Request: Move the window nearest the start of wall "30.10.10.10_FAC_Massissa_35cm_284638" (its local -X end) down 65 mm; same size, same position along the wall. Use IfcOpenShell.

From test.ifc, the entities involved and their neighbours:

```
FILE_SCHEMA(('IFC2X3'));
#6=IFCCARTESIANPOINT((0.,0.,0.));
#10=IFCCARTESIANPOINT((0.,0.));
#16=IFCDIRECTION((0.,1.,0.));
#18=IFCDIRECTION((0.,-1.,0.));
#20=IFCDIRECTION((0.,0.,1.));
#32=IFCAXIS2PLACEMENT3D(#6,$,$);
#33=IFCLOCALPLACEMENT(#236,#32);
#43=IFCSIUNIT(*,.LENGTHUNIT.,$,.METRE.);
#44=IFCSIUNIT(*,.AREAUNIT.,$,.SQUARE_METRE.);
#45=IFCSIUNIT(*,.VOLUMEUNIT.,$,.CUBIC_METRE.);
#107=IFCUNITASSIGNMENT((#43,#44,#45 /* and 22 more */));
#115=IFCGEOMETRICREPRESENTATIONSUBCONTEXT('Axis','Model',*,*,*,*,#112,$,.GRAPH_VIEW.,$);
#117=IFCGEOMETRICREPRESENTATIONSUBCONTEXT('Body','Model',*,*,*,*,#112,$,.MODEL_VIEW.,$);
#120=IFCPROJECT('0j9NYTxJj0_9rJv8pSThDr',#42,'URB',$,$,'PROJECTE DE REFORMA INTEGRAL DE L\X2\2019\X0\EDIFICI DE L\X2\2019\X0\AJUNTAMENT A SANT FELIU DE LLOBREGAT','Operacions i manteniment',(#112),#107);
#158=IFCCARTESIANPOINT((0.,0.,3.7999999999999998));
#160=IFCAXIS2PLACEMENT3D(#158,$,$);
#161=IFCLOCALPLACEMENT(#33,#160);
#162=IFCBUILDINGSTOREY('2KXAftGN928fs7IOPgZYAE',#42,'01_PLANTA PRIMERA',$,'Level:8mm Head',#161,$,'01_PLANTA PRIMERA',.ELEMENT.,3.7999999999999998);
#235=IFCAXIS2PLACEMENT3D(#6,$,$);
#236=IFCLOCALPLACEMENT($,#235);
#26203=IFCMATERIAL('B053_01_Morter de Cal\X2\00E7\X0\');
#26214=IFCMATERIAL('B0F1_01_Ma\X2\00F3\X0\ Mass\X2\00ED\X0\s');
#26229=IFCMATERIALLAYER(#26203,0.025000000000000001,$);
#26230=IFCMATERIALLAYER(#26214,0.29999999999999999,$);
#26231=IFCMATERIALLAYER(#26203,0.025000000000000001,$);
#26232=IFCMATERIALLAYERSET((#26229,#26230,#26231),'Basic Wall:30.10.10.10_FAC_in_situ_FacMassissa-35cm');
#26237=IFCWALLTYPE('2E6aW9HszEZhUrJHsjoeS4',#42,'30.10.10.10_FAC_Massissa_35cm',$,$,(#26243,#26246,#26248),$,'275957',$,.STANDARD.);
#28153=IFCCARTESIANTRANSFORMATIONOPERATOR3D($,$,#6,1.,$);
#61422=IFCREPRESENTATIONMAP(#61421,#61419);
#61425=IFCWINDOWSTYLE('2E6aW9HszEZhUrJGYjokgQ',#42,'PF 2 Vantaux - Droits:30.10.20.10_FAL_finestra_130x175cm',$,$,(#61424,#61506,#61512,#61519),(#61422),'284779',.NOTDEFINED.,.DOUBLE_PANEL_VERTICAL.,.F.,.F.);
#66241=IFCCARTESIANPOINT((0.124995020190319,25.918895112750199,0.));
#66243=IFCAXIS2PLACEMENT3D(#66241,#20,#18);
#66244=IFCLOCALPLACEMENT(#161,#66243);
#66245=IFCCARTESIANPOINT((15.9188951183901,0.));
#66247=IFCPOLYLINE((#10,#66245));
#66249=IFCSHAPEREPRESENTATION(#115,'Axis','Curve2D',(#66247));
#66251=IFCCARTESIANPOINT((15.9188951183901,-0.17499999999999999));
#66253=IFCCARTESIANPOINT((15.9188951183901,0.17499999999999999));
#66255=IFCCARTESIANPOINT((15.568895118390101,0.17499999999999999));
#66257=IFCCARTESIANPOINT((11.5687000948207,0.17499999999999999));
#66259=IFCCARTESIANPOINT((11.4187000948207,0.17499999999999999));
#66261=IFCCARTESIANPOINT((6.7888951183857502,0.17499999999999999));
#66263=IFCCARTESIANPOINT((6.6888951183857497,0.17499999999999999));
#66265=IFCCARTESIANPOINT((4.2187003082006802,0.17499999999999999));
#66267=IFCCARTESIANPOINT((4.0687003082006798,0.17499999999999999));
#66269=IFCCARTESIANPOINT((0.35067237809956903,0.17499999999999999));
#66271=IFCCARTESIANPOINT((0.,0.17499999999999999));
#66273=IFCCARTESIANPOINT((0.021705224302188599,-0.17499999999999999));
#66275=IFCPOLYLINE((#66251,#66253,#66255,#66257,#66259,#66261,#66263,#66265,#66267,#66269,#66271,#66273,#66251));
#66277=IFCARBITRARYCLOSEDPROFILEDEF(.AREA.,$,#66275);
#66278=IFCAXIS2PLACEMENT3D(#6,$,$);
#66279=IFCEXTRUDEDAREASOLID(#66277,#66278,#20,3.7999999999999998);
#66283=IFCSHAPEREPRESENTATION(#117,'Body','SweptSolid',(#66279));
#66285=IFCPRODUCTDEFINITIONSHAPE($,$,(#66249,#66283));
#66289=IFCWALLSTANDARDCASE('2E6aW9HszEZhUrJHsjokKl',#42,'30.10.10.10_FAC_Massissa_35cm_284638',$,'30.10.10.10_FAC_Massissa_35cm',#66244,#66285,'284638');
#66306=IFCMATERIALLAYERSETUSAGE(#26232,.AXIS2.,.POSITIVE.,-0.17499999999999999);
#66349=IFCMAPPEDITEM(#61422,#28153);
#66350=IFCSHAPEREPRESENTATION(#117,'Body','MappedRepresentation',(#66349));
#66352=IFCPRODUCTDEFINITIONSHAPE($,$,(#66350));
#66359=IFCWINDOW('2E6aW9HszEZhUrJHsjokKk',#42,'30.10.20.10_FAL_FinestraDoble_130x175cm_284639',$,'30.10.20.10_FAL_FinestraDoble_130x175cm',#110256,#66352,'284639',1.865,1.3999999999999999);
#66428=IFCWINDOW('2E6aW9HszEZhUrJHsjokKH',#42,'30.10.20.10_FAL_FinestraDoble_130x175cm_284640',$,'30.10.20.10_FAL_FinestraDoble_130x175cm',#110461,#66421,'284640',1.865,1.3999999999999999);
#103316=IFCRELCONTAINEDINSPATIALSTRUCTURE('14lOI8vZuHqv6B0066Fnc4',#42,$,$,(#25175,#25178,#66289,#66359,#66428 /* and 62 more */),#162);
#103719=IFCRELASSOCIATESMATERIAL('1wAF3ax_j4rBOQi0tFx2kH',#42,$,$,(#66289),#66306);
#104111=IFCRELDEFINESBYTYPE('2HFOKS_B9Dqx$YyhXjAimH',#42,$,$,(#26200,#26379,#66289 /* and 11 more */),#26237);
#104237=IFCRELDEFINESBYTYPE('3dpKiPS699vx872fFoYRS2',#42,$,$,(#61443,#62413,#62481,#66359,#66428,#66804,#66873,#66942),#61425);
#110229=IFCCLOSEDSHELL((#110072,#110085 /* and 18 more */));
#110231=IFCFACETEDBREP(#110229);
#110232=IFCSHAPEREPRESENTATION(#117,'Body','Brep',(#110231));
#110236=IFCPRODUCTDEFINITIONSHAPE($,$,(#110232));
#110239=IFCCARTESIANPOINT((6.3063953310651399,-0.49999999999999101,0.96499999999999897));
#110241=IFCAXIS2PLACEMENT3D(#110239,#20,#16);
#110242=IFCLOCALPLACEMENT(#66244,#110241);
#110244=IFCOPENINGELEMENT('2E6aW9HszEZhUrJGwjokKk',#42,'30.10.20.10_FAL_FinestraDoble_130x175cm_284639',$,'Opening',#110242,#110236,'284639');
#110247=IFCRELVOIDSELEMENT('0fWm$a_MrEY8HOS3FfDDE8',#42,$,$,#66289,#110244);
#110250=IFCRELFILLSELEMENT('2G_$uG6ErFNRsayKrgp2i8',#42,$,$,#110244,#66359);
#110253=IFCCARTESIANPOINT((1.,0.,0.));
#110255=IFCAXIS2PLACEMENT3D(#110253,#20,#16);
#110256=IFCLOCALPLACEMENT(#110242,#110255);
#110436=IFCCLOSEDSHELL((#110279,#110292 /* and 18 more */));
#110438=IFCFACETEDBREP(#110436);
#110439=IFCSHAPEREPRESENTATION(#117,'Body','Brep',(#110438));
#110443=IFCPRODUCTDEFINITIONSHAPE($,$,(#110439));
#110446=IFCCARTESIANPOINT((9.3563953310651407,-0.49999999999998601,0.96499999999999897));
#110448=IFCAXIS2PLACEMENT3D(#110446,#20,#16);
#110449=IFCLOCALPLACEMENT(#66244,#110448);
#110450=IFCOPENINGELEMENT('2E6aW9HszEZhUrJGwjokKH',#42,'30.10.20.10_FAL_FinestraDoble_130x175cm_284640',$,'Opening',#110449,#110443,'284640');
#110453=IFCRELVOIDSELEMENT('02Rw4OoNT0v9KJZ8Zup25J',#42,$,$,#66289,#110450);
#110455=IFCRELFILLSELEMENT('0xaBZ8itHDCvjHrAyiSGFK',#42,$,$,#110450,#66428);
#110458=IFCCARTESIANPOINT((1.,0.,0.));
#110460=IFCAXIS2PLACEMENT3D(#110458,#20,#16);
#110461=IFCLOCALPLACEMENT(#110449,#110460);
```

```python
import numpy as np
import ifcopenshell
import ifcopenshell.api.geometry
import ifcopenshell.util.placement
import ifcopenshell.util.unit

model = ifcopenshell.open("test.ifc")
unit_scale = ifcopenshell.util.unit.calculate_unit_scale(model)

window = model.by_guid("2E6aW9HszEZhUrJHsjokKk")
opening = window.FillsVoids[0].RelatingOpeningElement
dz = -0.065

shift = np.array([0.0, 0.0, dz])
# The window is placed relative to its opening, so it follows when the opening moves.
matrix = ifcopenshell.util.placement.get_local_placement(opening.ObjectPlacement)
matrix[:3, 3] += shift
ifcopenshell.api.geometry.edit_object_placement(
    model, product=opening, matrix=matrix, is_si=False, should_transform_children=True
)

print(f"moved by {dz * unit_scale:+.3f} m")

model.write("test_edited.ifc")
```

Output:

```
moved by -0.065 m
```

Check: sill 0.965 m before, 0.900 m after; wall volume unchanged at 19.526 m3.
